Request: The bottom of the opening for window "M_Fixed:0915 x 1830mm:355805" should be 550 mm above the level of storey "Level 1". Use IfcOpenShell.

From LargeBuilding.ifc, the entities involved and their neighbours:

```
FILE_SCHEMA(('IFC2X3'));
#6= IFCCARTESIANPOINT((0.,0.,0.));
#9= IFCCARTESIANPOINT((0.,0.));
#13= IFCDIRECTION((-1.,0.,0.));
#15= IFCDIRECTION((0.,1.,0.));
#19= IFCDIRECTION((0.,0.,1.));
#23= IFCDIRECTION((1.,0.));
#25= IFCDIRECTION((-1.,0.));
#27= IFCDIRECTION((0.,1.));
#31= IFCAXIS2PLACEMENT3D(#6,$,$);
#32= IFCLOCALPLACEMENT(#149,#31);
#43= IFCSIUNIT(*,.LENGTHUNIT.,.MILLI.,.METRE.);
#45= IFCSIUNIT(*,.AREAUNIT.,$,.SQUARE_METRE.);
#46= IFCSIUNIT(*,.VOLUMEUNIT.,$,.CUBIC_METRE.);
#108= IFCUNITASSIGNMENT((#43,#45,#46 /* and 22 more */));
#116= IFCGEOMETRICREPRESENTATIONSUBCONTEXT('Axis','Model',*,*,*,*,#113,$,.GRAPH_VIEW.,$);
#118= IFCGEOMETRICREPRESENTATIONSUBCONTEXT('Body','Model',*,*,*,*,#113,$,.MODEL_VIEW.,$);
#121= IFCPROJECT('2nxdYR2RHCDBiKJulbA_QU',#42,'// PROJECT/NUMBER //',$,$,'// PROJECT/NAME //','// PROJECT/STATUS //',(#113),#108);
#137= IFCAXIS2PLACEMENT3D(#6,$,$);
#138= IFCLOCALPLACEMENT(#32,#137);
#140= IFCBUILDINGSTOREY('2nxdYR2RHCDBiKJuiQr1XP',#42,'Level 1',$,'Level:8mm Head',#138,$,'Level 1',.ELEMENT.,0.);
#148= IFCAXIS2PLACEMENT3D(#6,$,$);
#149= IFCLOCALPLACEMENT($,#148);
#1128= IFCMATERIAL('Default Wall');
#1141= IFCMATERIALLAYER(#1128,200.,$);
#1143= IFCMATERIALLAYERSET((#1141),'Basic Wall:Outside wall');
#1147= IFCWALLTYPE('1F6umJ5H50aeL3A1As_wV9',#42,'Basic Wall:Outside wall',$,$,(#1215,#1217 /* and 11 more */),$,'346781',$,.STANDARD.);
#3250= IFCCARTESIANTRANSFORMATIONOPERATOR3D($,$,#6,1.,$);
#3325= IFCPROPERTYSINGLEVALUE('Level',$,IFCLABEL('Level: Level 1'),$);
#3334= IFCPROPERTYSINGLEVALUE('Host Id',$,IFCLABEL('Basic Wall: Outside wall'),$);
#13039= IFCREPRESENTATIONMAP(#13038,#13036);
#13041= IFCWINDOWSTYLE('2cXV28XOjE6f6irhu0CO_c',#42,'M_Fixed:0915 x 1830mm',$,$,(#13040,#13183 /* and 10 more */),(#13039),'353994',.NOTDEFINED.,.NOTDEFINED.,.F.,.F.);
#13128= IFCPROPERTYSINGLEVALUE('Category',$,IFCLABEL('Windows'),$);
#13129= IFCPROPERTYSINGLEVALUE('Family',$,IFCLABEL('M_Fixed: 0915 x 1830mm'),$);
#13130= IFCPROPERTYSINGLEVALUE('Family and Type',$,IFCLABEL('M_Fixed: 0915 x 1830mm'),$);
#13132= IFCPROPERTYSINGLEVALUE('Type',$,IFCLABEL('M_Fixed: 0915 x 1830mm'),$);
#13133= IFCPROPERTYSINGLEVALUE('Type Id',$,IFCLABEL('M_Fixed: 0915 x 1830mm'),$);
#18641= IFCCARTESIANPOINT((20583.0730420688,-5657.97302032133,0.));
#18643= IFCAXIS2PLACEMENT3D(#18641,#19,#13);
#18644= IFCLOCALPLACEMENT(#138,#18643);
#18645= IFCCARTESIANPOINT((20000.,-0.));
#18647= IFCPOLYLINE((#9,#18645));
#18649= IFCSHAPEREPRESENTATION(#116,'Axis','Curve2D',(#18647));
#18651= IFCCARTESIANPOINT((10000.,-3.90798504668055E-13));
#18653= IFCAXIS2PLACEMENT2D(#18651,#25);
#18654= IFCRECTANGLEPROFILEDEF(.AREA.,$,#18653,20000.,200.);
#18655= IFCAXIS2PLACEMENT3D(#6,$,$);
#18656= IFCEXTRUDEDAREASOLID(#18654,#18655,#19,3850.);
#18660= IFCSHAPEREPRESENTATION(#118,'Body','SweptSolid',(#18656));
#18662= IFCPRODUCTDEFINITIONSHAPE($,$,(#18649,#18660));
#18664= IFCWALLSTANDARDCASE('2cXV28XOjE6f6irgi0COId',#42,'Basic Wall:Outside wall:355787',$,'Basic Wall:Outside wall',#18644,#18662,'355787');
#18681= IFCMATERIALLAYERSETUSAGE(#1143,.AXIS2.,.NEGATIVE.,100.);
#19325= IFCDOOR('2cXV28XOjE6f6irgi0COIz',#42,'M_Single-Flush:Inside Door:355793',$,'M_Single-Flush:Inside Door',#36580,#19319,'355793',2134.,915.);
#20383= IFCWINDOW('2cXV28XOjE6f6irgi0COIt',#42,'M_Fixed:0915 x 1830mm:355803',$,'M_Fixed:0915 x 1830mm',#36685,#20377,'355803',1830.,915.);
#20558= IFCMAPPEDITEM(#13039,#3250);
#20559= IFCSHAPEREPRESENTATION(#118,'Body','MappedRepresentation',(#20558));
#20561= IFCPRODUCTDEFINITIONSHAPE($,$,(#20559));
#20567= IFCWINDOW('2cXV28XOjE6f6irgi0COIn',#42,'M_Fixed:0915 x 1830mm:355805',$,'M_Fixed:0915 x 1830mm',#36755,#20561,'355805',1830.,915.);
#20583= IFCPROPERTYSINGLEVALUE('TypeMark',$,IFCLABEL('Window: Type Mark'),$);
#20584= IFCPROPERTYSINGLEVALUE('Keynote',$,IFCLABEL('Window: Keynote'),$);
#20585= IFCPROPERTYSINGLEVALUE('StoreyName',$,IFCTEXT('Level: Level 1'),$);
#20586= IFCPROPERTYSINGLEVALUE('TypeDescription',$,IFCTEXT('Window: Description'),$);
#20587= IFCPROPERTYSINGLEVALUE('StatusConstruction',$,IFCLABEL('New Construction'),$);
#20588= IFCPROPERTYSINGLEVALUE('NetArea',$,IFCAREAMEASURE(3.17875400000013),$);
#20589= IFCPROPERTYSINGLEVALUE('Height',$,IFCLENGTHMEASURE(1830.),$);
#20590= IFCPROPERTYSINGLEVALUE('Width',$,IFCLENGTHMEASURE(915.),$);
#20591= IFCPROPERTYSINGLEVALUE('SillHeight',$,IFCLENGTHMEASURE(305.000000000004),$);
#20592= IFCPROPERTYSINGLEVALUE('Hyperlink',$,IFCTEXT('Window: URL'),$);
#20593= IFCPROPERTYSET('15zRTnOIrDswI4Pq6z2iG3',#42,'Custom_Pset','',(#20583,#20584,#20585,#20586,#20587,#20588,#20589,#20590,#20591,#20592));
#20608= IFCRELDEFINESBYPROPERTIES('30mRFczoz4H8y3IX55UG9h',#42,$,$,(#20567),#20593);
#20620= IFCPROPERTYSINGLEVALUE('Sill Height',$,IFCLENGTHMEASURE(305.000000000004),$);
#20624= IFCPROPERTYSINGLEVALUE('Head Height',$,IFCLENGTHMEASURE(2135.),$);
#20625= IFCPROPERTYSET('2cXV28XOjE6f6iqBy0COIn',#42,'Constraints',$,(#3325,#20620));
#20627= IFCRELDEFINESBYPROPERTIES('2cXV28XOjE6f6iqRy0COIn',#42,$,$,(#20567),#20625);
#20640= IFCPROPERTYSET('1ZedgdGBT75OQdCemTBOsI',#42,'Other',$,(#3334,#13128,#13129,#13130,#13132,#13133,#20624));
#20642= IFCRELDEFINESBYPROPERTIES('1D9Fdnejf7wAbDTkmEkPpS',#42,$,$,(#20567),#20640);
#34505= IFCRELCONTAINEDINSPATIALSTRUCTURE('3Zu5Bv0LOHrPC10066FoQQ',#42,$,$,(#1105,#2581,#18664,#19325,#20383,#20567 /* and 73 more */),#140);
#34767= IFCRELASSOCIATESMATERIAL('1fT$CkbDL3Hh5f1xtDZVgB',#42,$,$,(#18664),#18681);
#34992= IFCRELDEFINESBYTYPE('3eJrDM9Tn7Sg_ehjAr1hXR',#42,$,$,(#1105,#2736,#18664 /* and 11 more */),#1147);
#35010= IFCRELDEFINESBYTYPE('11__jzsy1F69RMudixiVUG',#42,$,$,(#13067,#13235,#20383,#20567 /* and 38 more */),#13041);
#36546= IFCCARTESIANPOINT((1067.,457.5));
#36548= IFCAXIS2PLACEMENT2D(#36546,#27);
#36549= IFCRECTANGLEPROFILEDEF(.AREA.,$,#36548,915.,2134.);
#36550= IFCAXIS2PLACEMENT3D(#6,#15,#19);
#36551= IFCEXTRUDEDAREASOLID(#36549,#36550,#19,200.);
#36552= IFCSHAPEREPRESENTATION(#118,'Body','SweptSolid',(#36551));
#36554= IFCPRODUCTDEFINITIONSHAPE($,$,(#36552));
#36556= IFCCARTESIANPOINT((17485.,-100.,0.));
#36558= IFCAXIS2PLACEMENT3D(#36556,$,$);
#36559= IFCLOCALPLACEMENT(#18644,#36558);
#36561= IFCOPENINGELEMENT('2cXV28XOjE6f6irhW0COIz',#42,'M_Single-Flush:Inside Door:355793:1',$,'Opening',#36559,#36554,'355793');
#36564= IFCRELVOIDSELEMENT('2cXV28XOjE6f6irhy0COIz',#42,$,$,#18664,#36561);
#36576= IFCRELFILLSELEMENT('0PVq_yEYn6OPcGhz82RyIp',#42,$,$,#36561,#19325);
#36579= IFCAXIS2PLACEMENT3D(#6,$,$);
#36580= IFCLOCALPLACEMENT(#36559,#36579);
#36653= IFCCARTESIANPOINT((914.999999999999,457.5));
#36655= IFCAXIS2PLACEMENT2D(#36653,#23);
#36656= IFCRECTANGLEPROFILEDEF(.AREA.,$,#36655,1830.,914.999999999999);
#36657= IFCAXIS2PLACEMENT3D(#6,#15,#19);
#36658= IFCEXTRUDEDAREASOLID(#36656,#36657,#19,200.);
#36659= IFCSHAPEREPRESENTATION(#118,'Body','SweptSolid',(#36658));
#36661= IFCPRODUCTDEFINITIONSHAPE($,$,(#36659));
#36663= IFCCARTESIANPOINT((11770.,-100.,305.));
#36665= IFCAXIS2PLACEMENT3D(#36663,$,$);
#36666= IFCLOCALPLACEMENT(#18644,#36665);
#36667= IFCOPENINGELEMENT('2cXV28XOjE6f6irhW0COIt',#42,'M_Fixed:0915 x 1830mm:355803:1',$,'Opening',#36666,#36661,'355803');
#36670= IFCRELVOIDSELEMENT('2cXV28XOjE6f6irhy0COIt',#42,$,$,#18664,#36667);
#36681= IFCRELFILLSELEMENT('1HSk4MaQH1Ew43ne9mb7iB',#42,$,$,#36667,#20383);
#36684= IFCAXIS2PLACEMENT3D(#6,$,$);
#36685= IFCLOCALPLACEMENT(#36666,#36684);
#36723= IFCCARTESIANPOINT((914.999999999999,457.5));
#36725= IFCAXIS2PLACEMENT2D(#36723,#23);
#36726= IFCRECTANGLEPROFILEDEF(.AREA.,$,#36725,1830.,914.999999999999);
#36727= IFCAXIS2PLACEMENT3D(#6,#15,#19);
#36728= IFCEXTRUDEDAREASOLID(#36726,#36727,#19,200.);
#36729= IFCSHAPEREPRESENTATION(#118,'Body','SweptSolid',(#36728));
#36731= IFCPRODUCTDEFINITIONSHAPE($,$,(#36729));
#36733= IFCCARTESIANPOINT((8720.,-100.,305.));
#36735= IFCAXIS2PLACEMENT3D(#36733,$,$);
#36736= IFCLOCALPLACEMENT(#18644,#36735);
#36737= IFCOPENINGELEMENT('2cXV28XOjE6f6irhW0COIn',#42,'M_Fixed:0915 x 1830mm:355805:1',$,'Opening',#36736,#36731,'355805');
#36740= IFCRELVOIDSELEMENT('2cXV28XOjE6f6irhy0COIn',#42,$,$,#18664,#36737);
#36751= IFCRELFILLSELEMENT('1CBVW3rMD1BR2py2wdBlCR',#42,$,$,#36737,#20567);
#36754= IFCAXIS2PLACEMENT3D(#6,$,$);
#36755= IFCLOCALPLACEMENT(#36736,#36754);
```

```python
import numpy as np
import ifcopenshell
import ifcopenshell.api.geometry
import ifcopenshell.api.pset
import ifcopenshell.geom
import ifcopenshell.util.element
import ifcopenshell.util.placement
import ifcopenshell.util.shape
import ifcopenshell.util.unit

model = ifcopenshell.open("LargeBuilding.ifc")
unit_scale = ifcopenshell.util.unit.calculate_unit_scale(model)

window = model.by_id(20567)
opening = window.FillsVoids[0].RelatingOpeningElement
storey = ifcopenshell.util.element.get_container(window, ifc_class="IfcBuildingStorey")
level = ifcopenshell.util.placement.get_local_placement(storey.ObjectPlacement)[2, 3]

# The opening's origin need not be at the sill, so measure its lowest point.
shape = ifcopenshell.geom.create_shape(ifcopenshell.geom.settings(), opening)
bottom = ifcopenshell.util.shape.get_shape_bottom_elevation(shape, shape.geometry) / unit_scale
dz = level + 550.0 - bottom

shift = np.array([0.0, 0.0, dz])
# The window is placed relative to its opening, so it follows when the opening moves.
matrix = ifcopenshell.util.placement.get_local_placement(opening.ObjectPlacement)
matrix[:3, 3] += shift
ifcopenshell.api.geometry.edit_object_placement(
    model, product=opening, matrix=matrix, is_si=False, should_transform_children=True
)

# Keep the stored heights in step.
pset = model.by_id(ifcopenshell.util.element.get_pset(window, "Custom_Pset", should_inherit=False)["id"])
ifcopenshell.api.pset.edit_pset(model, pset=pset, properties={
    "SillHeight": model.create_entity("IfcLengthMeasure", ifcopenshell.util.element.get_pset(window, "Constraints", "Sill Height") + dz),
})
pset = model.by_id(ifcopenshell.util.element.get_pset(window, "Constraints", should_inherit=False)["id"])
ifcopenshell.api.pset.edit_pset(model, pset=pset, properties={
    "Sill Height": model.create_entity("IfcLengthMeasure", ifcopenshell.util.element.get_pset(window, "Constraints", "Sill Height") + dz),
})
pset = model.by_id(ifcopenshell.util.element.get_pset(window, "Other", should_inherit=False)["id"])
ifcopenshell.api.pset.edit_pset(model, pset=pset, properties={
    "Head Height": model.create_entity("IfcLengthMeasure", ifcopenshell.util.element.get_pset(window, "Other", "Head Height") + dz),
})

print(f"moved by {dz * unit_scale:+.3f} m")

model.write("LargeBuilding_updated.ifc")
```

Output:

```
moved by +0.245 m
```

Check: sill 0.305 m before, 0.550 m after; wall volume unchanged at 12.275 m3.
